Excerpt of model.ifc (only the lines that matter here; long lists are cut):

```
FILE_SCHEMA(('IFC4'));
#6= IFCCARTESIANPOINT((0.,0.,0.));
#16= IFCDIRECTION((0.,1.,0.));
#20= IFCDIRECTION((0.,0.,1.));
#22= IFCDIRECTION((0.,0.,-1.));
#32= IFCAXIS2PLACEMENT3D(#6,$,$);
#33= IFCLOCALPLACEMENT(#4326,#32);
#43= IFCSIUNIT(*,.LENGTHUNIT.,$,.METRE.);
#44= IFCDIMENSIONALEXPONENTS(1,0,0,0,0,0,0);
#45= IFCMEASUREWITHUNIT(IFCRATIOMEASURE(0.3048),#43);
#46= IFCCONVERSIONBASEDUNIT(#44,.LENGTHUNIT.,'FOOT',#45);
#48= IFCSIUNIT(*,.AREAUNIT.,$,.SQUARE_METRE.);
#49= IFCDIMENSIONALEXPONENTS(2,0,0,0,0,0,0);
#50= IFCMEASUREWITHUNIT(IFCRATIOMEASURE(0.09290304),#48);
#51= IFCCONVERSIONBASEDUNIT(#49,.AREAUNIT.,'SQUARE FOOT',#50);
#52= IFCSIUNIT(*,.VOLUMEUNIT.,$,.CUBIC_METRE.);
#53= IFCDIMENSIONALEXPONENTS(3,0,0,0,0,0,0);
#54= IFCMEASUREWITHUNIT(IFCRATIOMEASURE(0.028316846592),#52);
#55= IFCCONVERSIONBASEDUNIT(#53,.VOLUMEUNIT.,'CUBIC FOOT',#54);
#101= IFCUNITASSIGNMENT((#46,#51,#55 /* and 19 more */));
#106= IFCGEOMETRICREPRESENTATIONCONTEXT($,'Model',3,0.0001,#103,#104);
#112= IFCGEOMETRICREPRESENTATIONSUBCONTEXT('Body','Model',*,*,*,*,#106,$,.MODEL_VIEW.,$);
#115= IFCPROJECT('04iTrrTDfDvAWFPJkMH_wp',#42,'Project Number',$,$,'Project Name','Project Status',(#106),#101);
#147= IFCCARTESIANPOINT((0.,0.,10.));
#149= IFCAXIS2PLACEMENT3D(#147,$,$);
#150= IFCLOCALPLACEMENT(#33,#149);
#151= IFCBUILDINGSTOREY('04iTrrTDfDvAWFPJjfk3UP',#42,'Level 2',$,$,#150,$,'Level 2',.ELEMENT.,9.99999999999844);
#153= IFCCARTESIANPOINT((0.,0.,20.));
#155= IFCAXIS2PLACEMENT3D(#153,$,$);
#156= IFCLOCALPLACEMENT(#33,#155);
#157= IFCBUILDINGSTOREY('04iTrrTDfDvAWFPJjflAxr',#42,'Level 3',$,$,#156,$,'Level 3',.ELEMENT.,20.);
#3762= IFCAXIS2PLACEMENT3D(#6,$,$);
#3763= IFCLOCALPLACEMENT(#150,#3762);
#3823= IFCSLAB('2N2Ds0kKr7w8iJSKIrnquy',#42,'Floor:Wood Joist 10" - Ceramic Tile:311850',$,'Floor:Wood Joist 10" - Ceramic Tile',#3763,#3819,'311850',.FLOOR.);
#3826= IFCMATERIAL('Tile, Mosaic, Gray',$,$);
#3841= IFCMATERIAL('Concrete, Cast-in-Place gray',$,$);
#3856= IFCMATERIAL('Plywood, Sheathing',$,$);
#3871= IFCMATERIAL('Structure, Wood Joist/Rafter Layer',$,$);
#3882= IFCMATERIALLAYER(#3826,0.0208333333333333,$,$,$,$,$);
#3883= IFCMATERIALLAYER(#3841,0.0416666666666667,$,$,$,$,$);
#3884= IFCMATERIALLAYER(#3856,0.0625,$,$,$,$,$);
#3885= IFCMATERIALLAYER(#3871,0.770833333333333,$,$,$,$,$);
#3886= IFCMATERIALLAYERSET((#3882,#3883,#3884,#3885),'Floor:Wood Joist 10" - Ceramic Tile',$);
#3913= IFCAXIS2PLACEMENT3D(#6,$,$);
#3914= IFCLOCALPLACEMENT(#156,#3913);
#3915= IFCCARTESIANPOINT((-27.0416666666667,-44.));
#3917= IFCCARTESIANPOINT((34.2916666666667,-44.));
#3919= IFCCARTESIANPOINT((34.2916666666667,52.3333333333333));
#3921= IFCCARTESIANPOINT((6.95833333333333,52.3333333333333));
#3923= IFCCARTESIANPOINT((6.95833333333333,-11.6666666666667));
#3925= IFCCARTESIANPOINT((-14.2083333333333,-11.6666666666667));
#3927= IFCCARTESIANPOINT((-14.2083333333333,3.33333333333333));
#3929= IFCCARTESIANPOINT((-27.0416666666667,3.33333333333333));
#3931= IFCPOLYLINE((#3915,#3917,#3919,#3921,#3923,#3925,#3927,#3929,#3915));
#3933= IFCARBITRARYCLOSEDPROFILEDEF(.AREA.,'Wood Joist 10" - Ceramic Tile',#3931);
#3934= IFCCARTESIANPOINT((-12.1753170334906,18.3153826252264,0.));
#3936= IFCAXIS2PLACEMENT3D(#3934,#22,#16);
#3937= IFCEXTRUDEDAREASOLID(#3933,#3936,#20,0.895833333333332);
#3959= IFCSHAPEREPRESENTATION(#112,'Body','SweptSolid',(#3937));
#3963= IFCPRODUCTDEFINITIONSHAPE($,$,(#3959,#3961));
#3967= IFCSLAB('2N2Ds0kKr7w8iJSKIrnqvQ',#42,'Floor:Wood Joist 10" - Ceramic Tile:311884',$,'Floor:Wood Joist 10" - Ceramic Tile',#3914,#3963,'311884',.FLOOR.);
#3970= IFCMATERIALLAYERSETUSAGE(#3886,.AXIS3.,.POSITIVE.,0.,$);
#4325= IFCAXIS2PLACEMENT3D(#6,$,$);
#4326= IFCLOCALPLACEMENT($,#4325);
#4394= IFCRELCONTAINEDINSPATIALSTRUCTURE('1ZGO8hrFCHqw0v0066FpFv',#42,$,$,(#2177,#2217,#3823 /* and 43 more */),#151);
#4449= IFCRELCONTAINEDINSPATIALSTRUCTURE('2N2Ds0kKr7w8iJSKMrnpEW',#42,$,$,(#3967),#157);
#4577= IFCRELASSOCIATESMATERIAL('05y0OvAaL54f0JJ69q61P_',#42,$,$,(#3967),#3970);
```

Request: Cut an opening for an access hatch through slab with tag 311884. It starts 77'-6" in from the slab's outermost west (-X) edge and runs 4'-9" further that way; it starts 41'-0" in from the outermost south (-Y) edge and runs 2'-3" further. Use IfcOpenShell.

```python
import numpy as np
import ifcopenshell
import ifcopenshell.api.feature
import ifcopenshell.api.geometry
import ifcopenshell.api.root
import ifcopenshell.geom
import ifcopenshell.util.placement
import ifcopenshell.util.representation
import ifcopenshell.util.shape
import ifcopenshell.util.unit

model = ifcopenshell.open("model.ifc")
unit_scale = ifcopenshell.util.unit.calculate_unit_scale(model)
settings = ifcopenshell.geom.settings()


def volume(element):
    """Net volume in cubic metres, openings subtracted."""
    shape = ifcopenshell.geom.create_shape(settings, element)
    return ifcopenshell.util.shape.get_volume(shape.geometry)


slab = model.by_guid("2N2Ds0kKr7w8iJSKIrnqvQ")
before = volume(slab)

# Extent in the slab's own axes, in metres. The edges named are its -X and -Y sides.
slab_shape = ifcopenshell.geom.create_shape(settings, slab)
vertices = ifcopenshell.util.shape.get_vertices(slab_shape.geometry)
x_min, y_min, bottom = vertices.min(axis=0)
top = vertices[:, 2].max()

opening = ifcopenshell.api.root.create_entity(model, ifc_class="IfcOpeningElement", name="Access hatch opening", predefined_type="OPENING")
context = ifcopenshell.util.representation.get_context(model, "Model", "Body", "MODEL_VIEW")
width, depth = 1.4478, 0.6858
outline = [(0.0, 0.0), (width, 0.0), (width, depth), (0.0, depth), (0.0, 0.0)]
# Overshoot both faces by 50 mm so the cut is clean.
shape = ifcopenshell.api.geometry.add_slab_representation(
    model, context=context, depth=top - bottom + 0.1, polyline=outline
)
ifcopenshell.api.geometry.assign_representation(model, product=opening, representation=shape)

matrix = ifcopenshell.util.placement.get_local_placement(slab.ObjectPlacement)
matrix[:, 3] = matrix @ np.append(np.array([x_min + 23.622, y_min + 12.4968, bottom - 0.05]) / unit_scale, 1.0)
ifcopenshell.api.geometry.edit_object_placement(model, product=opening, matrix=matrix, is_si=False)
ifcopenshell.api.feature.add_feature(model, feature=opening, element=slab)

after = volume(slab)

print(f"slab volume {before:.3f} -> {after:.3f} m3")

model.write("model-out.ifc")
```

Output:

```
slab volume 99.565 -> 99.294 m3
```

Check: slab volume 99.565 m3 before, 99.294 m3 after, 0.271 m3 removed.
